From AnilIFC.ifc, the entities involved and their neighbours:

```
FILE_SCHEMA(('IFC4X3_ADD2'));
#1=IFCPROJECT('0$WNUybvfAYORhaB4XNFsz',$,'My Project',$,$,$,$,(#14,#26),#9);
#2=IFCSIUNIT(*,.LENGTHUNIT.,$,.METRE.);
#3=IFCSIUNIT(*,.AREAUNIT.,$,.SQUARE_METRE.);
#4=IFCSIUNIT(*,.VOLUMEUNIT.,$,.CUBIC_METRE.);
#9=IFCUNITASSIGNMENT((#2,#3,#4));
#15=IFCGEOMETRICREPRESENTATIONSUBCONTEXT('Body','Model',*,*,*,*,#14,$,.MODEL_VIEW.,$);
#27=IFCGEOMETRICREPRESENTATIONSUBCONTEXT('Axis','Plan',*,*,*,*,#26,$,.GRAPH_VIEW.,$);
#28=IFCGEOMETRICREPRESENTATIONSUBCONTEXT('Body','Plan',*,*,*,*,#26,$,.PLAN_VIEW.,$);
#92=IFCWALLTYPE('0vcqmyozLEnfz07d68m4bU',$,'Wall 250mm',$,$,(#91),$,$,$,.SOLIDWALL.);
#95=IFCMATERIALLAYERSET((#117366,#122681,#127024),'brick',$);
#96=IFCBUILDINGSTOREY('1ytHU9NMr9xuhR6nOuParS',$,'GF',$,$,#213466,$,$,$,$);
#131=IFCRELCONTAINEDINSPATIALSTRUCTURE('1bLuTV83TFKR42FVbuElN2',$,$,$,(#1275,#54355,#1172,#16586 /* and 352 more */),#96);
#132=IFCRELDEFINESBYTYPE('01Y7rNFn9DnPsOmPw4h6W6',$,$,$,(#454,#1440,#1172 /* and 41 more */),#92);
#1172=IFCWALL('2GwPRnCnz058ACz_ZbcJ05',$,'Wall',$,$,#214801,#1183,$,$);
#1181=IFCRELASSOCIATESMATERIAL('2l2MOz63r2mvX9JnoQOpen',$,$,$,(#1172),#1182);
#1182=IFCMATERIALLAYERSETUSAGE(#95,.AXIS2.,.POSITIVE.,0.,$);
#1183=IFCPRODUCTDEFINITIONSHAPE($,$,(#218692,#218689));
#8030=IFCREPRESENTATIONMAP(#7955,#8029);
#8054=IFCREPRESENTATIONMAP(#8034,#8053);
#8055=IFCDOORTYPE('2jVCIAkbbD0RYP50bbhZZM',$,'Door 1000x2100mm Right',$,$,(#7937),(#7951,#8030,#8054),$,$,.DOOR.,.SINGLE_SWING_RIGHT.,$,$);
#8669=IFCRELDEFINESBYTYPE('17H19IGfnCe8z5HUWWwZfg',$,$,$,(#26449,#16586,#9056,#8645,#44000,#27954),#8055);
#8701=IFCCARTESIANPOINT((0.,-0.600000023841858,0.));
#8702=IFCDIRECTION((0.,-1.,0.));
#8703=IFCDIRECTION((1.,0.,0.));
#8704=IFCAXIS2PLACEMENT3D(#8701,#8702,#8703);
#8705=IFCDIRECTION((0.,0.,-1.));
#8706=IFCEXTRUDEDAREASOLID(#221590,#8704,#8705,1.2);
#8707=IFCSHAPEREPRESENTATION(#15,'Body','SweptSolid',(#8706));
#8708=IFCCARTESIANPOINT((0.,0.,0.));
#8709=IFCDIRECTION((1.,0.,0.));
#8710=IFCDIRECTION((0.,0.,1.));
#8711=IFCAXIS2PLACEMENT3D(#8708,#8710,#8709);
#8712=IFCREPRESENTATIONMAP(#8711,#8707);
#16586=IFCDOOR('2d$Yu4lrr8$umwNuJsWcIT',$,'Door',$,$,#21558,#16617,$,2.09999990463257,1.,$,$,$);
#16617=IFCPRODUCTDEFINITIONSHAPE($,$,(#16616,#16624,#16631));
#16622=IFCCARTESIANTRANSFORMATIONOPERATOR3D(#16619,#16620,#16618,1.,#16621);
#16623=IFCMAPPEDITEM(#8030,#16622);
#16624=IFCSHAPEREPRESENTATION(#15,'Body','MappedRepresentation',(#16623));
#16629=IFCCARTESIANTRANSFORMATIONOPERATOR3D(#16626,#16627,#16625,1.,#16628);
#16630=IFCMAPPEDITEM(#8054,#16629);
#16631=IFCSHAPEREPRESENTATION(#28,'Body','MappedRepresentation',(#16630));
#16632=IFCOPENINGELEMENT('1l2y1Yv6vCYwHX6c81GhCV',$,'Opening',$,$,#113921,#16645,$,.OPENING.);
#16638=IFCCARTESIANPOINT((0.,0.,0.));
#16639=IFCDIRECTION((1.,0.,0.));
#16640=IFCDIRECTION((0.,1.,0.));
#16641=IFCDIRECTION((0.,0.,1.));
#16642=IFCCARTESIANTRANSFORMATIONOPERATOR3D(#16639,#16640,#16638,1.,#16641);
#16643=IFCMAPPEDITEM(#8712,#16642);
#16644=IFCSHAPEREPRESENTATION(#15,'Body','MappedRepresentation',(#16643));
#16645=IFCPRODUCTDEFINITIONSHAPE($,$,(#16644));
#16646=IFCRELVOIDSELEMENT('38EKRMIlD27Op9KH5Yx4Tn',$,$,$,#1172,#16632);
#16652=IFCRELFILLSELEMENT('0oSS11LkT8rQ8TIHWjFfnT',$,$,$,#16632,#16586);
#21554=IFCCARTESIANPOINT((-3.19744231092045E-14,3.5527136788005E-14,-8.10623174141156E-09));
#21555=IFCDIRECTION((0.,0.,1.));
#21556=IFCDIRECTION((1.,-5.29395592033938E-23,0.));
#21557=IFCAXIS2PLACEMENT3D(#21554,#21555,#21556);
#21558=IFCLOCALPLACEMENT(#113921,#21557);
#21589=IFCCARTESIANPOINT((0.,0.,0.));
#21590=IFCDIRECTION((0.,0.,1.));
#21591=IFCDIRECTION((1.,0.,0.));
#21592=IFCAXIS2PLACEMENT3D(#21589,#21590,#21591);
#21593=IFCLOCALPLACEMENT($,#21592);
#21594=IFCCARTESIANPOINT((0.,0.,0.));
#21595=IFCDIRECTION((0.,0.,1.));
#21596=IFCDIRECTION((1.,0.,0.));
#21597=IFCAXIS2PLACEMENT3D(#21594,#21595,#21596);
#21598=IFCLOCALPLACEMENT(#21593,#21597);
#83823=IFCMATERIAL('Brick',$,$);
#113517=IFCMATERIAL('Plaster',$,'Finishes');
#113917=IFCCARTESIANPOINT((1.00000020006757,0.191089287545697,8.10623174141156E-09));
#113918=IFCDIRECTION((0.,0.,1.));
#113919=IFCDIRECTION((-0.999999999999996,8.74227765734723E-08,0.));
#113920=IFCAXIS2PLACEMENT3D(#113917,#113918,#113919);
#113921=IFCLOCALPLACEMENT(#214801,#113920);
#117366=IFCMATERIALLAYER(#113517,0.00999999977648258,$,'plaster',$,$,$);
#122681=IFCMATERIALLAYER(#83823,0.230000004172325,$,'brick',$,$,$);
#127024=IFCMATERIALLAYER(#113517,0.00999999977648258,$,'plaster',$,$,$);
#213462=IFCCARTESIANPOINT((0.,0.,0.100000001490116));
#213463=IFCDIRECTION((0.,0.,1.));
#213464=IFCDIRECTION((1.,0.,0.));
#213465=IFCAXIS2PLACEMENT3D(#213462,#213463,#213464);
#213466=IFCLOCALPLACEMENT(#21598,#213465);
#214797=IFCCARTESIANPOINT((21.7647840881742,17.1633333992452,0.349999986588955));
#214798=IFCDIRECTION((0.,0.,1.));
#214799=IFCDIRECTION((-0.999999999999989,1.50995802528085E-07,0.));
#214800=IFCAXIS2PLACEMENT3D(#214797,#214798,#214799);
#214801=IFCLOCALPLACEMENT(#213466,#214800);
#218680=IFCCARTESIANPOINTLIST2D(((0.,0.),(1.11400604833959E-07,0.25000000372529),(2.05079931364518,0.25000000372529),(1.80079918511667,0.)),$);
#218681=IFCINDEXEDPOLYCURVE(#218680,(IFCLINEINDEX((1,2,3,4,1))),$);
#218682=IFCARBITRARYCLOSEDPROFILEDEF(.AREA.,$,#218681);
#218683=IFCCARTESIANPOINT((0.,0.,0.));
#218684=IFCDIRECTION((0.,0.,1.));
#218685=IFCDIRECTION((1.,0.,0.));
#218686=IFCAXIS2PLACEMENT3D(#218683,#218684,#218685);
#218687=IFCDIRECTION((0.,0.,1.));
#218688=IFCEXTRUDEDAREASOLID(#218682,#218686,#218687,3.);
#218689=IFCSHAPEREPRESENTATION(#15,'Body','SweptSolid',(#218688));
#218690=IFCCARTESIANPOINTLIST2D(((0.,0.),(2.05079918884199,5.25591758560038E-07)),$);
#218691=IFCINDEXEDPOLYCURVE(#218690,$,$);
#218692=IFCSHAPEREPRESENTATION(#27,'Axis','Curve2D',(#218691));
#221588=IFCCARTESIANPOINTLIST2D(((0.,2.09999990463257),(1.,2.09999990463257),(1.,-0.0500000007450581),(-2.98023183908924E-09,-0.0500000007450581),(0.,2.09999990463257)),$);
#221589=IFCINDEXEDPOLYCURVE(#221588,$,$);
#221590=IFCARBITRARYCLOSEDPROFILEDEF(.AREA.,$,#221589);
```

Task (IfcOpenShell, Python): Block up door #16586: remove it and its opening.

```python
import ifcopenshell
import ifcopenshell.api.feature
import ifcopenshell.api.root
import ifcopenshell.geom
import ifcopenshell.util.shape

model = ifcopenshell.open("AnilIFC.ifc")
settings = ifcopenshell.geom.settings()


def volume(element):
    """Net volume in cubic metres, openings subtracted."""
    shape = ifcopenshell.geom.create_shape(settings, element)
    return ifcopenshell.util.shape.get_volume(shape.geometry)


door = model.by_guid("2d$Yu4lrr8$umwNuJsWcIT")
opening = door.FillsVoids[0].RelatingOpeningElement
wall = opening.VoidsElements[0].RelatingBuildingElement
before = volume(wall)

ifcopenshell.api.root.remove_product(model, product=door)
ifcopenshell.api.feature.remove_feature(model, feature=opening)

after = volume(wall)

print(f"wall volume {before:.3f} -> {after:.3f} m3")

model.write("AnilIFC-out.ifc")
```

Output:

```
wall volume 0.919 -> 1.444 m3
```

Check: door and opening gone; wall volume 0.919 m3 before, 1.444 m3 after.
